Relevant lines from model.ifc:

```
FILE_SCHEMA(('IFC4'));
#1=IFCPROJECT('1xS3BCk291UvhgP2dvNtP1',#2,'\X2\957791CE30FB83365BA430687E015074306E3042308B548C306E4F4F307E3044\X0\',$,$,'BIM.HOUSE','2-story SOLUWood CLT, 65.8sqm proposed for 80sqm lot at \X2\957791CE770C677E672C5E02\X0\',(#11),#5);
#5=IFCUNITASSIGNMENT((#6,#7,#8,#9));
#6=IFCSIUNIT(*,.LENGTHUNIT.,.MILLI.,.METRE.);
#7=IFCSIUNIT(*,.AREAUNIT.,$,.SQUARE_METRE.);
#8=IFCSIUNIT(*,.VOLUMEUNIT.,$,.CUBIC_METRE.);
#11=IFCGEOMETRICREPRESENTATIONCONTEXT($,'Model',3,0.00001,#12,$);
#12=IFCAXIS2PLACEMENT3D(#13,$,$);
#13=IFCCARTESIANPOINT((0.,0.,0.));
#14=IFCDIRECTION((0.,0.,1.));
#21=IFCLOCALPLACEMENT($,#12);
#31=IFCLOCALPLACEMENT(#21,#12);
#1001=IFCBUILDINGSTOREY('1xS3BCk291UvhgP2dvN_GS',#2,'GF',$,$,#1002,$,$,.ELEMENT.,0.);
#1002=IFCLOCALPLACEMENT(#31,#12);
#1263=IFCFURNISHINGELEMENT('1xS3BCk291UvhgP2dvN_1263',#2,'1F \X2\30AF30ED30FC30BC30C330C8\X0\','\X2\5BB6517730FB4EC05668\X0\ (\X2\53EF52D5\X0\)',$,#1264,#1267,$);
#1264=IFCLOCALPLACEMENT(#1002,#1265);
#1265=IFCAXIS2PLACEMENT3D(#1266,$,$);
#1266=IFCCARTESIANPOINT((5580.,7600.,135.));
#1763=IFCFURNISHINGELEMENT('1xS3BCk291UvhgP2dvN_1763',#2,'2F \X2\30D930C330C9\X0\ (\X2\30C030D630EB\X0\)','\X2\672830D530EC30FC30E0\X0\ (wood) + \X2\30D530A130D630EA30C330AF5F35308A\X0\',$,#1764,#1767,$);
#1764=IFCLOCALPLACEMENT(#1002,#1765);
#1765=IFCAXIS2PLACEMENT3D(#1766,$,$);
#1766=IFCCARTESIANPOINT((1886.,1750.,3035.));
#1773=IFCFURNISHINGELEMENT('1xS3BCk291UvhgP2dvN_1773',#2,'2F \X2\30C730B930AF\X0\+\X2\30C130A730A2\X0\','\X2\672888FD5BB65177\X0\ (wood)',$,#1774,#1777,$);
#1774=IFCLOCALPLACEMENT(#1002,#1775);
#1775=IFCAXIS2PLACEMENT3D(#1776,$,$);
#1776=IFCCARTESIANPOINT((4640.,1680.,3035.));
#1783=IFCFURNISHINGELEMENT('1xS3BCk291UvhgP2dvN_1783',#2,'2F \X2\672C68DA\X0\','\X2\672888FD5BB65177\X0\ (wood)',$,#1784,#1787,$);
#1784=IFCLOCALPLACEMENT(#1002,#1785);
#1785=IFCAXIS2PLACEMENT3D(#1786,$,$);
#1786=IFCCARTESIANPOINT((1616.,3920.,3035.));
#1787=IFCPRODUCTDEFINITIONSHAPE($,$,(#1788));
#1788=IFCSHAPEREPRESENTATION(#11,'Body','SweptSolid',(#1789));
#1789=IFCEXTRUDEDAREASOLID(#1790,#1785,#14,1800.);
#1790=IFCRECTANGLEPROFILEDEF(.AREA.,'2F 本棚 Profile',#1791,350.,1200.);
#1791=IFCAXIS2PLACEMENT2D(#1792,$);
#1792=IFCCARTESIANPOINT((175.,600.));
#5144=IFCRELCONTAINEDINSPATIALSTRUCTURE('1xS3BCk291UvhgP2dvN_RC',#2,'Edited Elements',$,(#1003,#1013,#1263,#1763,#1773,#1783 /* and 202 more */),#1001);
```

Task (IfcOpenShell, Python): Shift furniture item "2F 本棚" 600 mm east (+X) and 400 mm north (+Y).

```python
import ifcopenshell
import ifcopenshell.api.geometry
import ifcopenshell.util.placement
import ifcopenshell.util.unit

model = ifcopenshell.open("model.ifc")
unit_scale = ifcopenshell.util.unit.calculate_unit_scale(model)

item = model.by_id(1783)
matrix = ifcopenshell.util.placement.get_local_placement(item.ObjectPlacement)
matrix[0, 3] += 0.6 / unit_scale
matrix[1, 3] += 0.4 / unit_scale
ifcopenshell.api.geometry.edit_object_placement(model, product=item, matrix=matrix, is_si=False)

print(ifcopenshell.util.placement.get_local_placement(item.ObjectPlacement).round(3) + 0.0)

model.write("model_rev.ifc")
```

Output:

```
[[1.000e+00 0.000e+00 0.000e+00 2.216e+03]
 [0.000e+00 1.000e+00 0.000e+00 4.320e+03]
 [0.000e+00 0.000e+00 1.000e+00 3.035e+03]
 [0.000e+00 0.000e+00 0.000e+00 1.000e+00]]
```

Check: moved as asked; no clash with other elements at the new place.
